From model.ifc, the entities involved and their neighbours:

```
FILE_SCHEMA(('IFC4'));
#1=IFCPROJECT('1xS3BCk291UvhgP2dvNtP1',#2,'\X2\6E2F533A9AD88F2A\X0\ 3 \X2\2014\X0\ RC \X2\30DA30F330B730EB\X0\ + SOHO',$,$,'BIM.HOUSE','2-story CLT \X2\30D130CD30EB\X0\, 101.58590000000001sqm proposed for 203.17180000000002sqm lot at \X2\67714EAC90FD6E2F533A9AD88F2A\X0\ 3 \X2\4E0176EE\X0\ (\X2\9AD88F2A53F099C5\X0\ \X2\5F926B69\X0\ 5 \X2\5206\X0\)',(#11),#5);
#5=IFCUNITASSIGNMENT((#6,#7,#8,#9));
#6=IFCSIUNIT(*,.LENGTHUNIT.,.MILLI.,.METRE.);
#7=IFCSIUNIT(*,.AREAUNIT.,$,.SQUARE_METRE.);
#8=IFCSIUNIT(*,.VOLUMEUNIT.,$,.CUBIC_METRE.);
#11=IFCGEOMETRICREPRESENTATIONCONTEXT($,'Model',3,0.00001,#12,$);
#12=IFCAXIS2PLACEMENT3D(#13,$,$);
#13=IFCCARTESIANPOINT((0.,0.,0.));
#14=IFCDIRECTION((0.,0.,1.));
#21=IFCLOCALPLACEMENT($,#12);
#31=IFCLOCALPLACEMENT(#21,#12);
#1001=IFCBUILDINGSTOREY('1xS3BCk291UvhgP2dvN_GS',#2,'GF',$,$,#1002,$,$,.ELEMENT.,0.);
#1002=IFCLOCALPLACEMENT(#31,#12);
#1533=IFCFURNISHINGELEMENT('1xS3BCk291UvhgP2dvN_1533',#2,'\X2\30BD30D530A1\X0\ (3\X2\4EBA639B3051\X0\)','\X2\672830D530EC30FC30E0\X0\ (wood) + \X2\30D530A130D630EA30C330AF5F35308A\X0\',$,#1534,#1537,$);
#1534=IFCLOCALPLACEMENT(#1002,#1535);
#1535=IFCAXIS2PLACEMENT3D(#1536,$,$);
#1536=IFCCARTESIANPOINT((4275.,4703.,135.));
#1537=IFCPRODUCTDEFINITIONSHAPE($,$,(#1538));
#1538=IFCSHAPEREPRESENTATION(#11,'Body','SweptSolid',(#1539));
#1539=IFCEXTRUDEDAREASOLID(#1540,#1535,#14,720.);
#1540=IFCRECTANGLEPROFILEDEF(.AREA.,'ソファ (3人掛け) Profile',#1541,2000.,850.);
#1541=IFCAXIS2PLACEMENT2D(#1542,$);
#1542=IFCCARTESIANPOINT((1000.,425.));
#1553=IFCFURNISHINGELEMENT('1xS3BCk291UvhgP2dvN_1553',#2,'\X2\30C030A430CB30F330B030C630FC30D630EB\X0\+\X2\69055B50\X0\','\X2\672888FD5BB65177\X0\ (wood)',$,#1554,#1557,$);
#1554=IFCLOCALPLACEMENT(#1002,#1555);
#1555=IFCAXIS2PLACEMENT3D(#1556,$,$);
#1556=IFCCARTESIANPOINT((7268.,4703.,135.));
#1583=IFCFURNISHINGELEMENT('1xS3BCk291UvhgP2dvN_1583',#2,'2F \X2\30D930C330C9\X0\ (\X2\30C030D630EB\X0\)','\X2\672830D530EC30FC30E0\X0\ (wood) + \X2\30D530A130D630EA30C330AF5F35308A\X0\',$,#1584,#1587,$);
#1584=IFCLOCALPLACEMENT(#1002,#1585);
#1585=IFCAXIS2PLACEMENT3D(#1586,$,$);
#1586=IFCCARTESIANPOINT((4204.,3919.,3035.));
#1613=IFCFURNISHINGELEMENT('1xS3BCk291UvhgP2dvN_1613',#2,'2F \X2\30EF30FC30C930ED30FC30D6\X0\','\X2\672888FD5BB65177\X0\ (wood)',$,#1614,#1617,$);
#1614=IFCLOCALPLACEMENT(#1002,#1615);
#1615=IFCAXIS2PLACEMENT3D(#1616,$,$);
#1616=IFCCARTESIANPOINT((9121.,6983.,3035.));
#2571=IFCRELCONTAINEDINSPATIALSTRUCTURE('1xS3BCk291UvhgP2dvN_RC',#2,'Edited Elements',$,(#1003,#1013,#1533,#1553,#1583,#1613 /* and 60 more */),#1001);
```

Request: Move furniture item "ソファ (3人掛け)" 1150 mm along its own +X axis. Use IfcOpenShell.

```python
import ifcopenshell
import ifcopenshell.api.geometry
import ifcopenshell.util.placement

model = ifcopenshell.open("model.ifc")

item = model.by_guid("1xS3BCk291UvhgP2dvN_1533")
matrix = ifcopenshell.util.placement.get_local_placement(item.ObjectPlacement)
matrix[:3, 3] += matrix[:3, 0] * 1150.0
ifcopenshell.api.geometry.edit_object_placement(model, product=item, matrix=matrix, is_si=False)

print(ifcopenshell.util.placement.get_local_placement(item.ObjectPlacement).round(3) + 0.0)

model.write("model_updated.ifc")
```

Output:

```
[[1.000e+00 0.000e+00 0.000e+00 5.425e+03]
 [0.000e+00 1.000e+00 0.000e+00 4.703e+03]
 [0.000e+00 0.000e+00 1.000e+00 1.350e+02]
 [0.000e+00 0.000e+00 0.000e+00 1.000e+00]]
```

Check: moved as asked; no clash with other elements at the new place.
